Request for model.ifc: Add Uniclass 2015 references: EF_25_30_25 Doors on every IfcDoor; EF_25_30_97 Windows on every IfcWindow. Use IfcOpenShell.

First a look at what the model holds.

```python
import ifcopenshell

model = ifcopenshell.open("model.ifc")
print(model.schema)
print("classifications:", [c.Name for c in model.by_type("IfcClassification")])
for ifc_class in ("IfcDoor", "IfcRoof", "IfcStair", "IfcWall", "IfcWindow"):
    print(ifc_class, len(model.by_type(ifc_class)))
```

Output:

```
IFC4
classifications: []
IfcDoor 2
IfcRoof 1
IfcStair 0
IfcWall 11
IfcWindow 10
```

```python
import ifcopenshell
import ifcopenshell.api.classification

model = ifcopenshell.open("model.ifc")

system = ifcopenshell.api.classification.add_classification(model, classification="Uniclass 2015")

codes = {
    "IfcDoor": ("EF_25_30_25", "Doors"),
    "IfcWindow": ("EF_25_30_97", "Windows"),
}
for ifc_class, (code, name) in codes.items():
    products = model.by_type(ifc_class)
    ifcopenshell.api.classification.add_reference(
        model, products=products, classification=system, identification=code, name=name
    )
    print(code, len(products))

model.write("model_edited.ifc")
```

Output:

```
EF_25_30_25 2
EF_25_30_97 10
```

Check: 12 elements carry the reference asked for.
